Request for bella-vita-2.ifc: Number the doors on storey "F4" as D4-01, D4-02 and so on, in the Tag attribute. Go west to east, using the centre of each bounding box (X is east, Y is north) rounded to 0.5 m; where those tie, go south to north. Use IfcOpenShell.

First a look at what the model holds.

```python
import ifcopenshell
import ifcopenshell.util.element
import ifcopenshell.util.placement

model = ifcopenshell.open("bella-vita-2.ifc")
print(model.schema)
storey = next(s for s in model.by_type("IfcBuildingStorey") if s.Name == "F4")
doors = [e for e in ifcopenshell.util.element.get_decomposition(storey) if e.is_a("IfcDoor")]
for e in sorted(doors, key=lambda e: e.id()):
    origin = ifcopenshell.util.placement.get_local_placement(e.ObjectPlacement)[:3, 3]
    print(e.id(), e.Tag, e.Name, origin.round(2) + 0.0, sep=" | ")
```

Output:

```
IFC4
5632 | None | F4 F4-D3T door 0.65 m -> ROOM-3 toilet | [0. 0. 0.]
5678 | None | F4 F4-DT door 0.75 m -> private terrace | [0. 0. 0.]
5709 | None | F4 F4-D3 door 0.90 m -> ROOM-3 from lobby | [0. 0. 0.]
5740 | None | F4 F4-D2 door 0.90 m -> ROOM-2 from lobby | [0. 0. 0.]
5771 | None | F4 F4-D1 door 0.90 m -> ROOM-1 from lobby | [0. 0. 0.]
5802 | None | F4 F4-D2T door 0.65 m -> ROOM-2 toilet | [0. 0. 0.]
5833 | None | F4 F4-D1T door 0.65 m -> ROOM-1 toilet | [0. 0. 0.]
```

```python
import ifcopenshell
import ifcopenshell.geom
import ifcopenshell.util.element
import ifcopenshell.util.shape

model = ifcopenshell.open("bella-vita-2.ifc")
settings = ifcopenshell.geom.settings()
settings.set("use-world-coords", True)


def centre(element):
    shape = ifcopenshell.geom.create_shape(settings, element)
    return ifcopenshell.util.shape.get_bbox_centroid(shape.geometry)


storey = next(s for s in model.by_type("IfcBuildingStorey") if s.Name == "F4")
doors = [e for e in ifcopenshell.util.element.get_decomposition(storey) if e.is_a("IfcDoor")]

# Insertion points can sit at a corner or the storey origin, so sort by the geometry (in metres).
centres = {e: centre(e) for e in doors}
doors.sort(key=lambda e: (round(centres[e][0] / 0.5), centres[e][1]))

for i, e in enumerate(doors, start=1):
    number = f"D4-{i:02d}"
    e.Tag = number
    print(e.id(), number)

model.write("bella-vita-2_v2.ifc")
```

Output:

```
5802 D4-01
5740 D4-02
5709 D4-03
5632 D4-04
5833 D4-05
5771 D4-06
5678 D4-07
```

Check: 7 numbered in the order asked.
